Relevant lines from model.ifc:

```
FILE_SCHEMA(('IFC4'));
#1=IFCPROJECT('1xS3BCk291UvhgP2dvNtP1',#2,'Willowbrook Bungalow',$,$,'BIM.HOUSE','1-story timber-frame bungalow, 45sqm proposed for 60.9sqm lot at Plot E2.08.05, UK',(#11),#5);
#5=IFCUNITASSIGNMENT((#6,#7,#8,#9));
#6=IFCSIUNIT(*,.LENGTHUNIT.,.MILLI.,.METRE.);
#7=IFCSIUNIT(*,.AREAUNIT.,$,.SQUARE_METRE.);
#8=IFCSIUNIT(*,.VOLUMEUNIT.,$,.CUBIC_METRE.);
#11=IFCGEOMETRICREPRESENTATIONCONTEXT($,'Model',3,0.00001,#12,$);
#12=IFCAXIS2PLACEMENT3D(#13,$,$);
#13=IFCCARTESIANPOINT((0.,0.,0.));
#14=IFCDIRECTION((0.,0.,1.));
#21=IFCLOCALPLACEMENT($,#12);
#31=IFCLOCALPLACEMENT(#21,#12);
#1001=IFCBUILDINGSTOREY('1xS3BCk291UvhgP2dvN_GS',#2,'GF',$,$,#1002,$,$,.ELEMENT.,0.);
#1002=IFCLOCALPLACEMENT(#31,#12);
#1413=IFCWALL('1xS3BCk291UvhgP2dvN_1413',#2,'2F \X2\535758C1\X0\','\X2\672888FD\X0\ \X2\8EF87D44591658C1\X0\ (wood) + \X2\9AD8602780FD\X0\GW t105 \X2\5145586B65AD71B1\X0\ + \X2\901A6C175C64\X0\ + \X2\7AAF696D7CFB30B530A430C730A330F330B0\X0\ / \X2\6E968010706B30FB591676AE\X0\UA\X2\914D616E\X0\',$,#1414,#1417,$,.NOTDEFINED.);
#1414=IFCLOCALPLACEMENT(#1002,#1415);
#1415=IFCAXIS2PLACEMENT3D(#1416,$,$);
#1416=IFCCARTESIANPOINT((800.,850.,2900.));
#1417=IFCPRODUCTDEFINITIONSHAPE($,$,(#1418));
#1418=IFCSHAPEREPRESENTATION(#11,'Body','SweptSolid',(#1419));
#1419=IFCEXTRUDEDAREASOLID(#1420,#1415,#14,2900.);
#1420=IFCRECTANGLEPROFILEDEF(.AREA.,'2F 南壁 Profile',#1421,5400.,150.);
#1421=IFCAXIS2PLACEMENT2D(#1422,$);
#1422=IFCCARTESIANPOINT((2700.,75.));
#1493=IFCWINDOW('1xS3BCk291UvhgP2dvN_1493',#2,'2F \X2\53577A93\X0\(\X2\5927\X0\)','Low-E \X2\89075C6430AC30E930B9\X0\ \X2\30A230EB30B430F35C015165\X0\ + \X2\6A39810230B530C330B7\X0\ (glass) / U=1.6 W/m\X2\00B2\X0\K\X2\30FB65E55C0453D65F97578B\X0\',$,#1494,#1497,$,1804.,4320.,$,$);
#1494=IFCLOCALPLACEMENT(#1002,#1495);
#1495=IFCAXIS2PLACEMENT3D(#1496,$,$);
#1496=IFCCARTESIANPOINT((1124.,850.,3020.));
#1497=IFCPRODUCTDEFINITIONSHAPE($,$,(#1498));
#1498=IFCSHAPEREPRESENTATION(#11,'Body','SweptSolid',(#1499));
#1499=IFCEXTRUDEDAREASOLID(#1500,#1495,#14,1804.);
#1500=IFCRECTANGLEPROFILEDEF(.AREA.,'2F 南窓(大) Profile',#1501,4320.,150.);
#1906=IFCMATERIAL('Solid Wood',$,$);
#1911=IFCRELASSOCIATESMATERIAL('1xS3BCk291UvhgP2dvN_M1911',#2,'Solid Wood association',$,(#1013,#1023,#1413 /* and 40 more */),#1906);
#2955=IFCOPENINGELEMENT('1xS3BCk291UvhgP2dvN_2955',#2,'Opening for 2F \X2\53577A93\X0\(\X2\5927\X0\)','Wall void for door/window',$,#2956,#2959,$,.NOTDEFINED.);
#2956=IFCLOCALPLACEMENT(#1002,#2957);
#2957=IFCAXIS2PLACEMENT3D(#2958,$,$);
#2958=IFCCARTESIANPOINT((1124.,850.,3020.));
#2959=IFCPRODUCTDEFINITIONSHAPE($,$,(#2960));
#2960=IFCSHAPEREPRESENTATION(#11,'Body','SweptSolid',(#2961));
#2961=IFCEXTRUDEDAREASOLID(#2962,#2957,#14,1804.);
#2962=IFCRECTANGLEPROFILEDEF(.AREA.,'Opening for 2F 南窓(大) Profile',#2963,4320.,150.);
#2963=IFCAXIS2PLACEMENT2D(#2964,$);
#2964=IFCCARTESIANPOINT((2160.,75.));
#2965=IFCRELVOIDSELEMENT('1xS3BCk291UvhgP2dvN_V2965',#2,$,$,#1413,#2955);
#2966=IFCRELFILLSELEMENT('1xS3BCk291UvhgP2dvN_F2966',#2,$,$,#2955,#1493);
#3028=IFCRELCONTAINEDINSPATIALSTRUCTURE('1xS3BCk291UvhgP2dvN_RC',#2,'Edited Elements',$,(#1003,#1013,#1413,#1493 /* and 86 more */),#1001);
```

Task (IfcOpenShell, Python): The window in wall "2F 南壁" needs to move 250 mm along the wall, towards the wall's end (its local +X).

```python
import ifcopenshell
import ifcopenshell.api.geometry
import ifcopenshell.util.placement
import ifcopenshell.util.unit

model = ifcopenshell.open("model.ifc")
unit_scale = ifcopenshell.util.unit.calculate_unit_scale(model)

window = model.by_guid("1xS3BCk291UvhgP2dvN_1493")
opening = window.FillsVoids[0].RelatingOpeningElement
wall = opening.VoidsElements[0].RelatingBuildingElement

wall_matrix = ifcopenshell.util.placement.get_local_placement(wall.ObjectPlacement)
shift = wall_matrix[:3, 0] * 0.25 / unit_scale
before = ifcopenshell.util.placement.get_local_placement(window.ObjectPlacement)[:3, 3].copy()

# The window is not placed relative to its opening, so move both.
for product in (opening, window):
    matrix = ifcopenshell.util.placement.get_local_placement(product.ObjectPlacement)
    matrix[:3, 3] += shift
    ifcopenshell.api.geometry.edit_object_placement(model, product=product, matrix=matrix, is_si=False)

after = ifcopenshell.util.placement.get_local_placement(window.ObjectPlacement)[:3, 3]
print("window moved by", (after - before).round(3) + 0.0)

model.write("model_updated.ifc")
```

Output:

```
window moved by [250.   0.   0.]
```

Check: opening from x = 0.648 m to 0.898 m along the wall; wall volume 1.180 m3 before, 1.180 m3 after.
